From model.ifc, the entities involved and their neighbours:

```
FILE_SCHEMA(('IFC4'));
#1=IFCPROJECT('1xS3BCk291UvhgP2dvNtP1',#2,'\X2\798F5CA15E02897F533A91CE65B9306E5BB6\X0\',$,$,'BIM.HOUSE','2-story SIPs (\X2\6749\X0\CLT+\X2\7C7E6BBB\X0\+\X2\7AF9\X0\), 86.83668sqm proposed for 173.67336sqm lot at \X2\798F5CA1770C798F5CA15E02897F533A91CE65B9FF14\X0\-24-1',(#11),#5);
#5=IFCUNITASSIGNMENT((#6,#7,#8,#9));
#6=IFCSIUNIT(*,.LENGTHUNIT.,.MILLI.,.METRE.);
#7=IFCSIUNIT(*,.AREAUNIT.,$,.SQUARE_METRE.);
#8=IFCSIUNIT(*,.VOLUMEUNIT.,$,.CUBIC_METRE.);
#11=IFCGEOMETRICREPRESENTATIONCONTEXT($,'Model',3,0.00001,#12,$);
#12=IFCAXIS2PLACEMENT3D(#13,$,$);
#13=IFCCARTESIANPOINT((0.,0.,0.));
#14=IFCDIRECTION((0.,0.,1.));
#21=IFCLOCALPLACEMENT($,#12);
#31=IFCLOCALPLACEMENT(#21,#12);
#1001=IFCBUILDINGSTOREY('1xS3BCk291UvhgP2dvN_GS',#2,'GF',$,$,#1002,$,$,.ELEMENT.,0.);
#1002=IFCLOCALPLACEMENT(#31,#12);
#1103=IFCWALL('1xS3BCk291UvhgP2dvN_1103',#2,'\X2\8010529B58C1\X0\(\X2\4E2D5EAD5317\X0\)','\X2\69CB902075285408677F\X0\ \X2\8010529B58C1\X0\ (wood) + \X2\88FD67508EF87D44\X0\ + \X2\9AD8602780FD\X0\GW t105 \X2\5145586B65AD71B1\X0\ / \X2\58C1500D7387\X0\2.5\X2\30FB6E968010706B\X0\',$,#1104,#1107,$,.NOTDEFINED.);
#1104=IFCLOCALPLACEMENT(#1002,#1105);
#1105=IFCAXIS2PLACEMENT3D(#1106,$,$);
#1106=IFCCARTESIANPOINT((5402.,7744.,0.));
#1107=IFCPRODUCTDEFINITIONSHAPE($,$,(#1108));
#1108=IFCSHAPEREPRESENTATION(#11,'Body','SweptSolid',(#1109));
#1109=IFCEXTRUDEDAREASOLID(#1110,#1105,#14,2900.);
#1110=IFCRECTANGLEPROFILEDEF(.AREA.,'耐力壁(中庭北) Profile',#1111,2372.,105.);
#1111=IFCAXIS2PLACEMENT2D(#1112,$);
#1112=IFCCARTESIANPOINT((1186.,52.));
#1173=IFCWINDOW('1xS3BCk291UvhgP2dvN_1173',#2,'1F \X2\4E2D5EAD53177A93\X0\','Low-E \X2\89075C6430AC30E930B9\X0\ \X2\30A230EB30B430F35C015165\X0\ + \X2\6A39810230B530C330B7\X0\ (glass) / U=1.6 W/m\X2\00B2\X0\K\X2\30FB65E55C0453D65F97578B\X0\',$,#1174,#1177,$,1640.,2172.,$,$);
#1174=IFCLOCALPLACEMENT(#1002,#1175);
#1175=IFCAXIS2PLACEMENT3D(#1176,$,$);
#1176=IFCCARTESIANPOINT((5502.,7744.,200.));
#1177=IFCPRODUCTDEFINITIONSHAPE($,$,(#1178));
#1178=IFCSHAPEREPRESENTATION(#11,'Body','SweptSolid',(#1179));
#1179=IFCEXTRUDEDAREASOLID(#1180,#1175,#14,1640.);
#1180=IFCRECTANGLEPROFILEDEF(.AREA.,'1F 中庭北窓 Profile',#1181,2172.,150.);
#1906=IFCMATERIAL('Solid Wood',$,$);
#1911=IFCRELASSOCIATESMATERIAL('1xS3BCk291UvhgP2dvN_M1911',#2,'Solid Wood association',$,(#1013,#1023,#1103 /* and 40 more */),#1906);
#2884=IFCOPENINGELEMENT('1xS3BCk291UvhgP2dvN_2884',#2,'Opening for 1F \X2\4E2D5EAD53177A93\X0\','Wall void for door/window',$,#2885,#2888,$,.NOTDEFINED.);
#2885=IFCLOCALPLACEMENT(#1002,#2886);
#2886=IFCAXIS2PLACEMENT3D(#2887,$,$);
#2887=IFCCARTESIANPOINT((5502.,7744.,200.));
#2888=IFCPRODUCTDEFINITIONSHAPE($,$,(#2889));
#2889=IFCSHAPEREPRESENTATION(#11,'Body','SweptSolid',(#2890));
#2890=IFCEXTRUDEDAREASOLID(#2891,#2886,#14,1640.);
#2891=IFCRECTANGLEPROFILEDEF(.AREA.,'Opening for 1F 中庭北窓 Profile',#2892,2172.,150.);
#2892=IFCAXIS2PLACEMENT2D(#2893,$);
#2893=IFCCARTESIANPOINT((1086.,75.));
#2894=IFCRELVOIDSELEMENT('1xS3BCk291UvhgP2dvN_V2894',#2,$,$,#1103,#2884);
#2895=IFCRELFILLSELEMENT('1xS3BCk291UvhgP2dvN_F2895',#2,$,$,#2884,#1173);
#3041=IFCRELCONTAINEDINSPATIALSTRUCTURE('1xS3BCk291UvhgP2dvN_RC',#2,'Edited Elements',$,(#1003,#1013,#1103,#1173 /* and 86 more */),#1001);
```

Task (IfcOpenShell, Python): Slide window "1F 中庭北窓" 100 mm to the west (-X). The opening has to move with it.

```python
import ifcopenshell
import ifcopenshell.api.geometry
import ifcopenshell.util.placement

model = ifcopenshell.open("model.ifc")

window = model.by_guid("1xS3BCk291UvhgP2dvN_1173")
opening = window.FillsVoids[0].RelatingOpeningElement
wall = opening.VoidsElements[0].RelatingBuildingElement

wall_matrix = ifcopenshell.util.placement.get_local_placement(wall.ObjectPlacement)
shift = wall_matrix[:3, 0] * -100.0
before = ifcopenshell.util.placement.get_local_placement(window.ObjectPlacement)[:3, 3].copy()

# The window is not placed relative to its opening, so move both.
for product in (opening, window):
    matrix = ifcopenshell.util.placement.get_local_placement(product.ObjectPlacement)
    matrix[:3, 3] += shift
    ifcopenshell.api.geometry.edit_object_placement(model, product=product, matrix=matrix, is_si=False)

after = ifcopenshell.util.placement.get_local_placement(window.ObjectPlacement)[:3, 3]
print("window moved by", (after - before).round(3) + 0.0)

model.write("model_updated.ifc")
```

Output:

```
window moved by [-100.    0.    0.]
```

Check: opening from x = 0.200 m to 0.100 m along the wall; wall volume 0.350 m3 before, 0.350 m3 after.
